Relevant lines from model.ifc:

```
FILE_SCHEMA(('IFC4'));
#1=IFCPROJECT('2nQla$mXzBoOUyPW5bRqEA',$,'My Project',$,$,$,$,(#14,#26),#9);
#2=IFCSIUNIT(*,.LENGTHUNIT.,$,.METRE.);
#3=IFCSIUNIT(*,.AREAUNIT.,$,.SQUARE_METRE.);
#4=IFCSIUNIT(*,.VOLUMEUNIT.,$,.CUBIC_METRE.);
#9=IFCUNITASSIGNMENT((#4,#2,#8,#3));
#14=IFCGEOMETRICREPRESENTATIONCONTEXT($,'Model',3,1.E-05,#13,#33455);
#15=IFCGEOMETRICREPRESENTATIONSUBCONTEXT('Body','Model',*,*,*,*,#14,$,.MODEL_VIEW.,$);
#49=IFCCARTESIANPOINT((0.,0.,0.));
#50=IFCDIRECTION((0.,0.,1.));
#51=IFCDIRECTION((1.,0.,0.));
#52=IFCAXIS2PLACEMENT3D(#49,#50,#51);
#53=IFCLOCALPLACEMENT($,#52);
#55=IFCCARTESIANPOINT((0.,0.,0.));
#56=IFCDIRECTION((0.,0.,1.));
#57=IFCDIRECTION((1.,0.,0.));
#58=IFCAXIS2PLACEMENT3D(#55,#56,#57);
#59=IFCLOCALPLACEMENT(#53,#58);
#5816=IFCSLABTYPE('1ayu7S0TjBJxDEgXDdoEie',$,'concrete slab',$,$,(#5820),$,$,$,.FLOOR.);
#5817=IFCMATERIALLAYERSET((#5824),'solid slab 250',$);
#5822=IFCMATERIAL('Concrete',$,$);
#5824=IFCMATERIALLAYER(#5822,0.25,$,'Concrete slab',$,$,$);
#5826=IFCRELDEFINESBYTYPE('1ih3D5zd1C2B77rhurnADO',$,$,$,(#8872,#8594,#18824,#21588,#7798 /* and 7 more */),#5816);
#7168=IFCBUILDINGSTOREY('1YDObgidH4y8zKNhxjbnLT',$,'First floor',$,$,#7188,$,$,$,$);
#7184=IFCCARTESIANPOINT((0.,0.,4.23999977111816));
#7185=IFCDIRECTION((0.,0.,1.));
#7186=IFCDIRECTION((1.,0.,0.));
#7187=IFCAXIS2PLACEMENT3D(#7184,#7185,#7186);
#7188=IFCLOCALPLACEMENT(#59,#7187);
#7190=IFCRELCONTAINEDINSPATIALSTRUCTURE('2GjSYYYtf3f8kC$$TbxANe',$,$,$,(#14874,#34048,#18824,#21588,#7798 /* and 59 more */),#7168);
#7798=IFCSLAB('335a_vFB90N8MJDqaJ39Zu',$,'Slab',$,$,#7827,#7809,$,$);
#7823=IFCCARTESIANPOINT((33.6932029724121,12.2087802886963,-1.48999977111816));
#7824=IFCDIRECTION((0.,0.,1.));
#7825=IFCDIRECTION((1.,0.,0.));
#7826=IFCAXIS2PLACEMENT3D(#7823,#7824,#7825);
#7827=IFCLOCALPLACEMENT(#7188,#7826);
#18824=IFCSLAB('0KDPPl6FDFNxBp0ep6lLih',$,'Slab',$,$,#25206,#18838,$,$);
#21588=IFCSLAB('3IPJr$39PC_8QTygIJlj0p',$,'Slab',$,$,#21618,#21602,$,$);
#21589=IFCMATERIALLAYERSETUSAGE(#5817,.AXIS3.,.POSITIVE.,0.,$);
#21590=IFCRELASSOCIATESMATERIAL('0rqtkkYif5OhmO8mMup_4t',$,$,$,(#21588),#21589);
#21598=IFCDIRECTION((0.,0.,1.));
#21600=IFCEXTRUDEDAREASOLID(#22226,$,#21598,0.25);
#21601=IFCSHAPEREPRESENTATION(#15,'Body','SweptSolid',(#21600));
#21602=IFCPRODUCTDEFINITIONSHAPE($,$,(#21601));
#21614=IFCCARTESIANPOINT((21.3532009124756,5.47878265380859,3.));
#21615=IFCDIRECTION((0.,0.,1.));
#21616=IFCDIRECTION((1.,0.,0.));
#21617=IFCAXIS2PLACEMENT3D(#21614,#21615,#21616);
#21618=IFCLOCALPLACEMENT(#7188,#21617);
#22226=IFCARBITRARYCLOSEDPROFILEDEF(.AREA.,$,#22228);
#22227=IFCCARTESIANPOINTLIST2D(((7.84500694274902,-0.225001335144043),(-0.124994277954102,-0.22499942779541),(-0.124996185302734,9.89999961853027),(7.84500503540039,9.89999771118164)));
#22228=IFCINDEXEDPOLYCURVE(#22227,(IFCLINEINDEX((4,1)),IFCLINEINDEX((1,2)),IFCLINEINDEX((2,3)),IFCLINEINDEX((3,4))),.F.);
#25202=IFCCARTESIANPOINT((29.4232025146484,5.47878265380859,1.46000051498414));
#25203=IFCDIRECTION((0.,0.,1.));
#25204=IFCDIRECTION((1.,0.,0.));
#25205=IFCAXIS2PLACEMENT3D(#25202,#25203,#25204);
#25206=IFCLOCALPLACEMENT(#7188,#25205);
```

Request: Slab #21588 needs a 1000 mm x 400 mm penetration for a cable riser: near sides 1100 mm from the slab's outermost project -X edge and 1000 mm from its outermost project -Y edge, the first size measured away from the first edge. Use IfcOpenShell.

```python
import numpy as np
import ifcopenshell
import ifcopenshell.api.feature
import ifcopenshell.api.geometry
import ifcopenshell.api.root
import ifcopenshell.geom
import ifcopenshell.util.placement
import ifcopenshell.util.representation
import ifcopenshell.util.shape
import ifcopenshell.util.unit

model = ifcopenshell.open("model.ifc")
unit_scale = ifcopenshell.util.unit.calculate_unit_scale(model)
settings = ifcopenshell.geom.settings()


def volume(element):
    """Net volume in cubic metres, openings subtracted."""
    shape = ifcopenshell.geom.create_shape(settings, element)
    return ifcopenshell.util.shape.get_volume(shape.geometry)


slab = model.by_id(21588)
before = volume(slab)

# Extent in the slab's own axes, in metres. The edges named are its -X and -Y sides.
slab_shape = ifcopenshell.geom.create_shape(settings, slab)
vertices = ifcopenshell.util.shape.get_vertices(slab_shape.geometry)
x_min, y_min, bottom = vertices.min(axis=0)
top = vertices[:, 2].max()

opening = ifcopenshell.api.root.create_entity(model, ifc_class="IfcOpeningElement", name="Cable riser opening", predefined_type="OPENING")
context = ifcopenshell.util.representation.get_context(model, "Model", "Body", "MODEL_VIEW")
width, depth = 1, 0.4
outline = [(0.0, 0.0), (width, 0.0), (width, depth), (0.0, depth), (0.0, 0.0)]
# Overshoot both faces by 50 mm so the cut is clean.
shape = ifcopenshell.api.geometry.add_slab_representation(
    model, context=context, depth=top - bottom + 0.1, polyline=outline
)
ifcopenshell.api.geometry.assign_representation(model, product=opening, representation=shape)

matrix = ifcopenshell.util.placement.get_local_placement(slab.ObjectPlacement)
matrix[:, 3] = matrix @ np.append(np.array([x_min + 1.1, y_min + 1, bottom - 0.05]) / unit_scale, 1.0)
ifcopenshell.api.geometry.edit_object_placement(model, product=opening, matrix=matrix, is_si=False)
ifcopenshell.api.feature.add_feature(model, feature=opening, element=slab)

after = volume(slab)

print(f"slab volume {before:.3f} -> {after:.3f} m3")

model.write("model_v2.ifc")
```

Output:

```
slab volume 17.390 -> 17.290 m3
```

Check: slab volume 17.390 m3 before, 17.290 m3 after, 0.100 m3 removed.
